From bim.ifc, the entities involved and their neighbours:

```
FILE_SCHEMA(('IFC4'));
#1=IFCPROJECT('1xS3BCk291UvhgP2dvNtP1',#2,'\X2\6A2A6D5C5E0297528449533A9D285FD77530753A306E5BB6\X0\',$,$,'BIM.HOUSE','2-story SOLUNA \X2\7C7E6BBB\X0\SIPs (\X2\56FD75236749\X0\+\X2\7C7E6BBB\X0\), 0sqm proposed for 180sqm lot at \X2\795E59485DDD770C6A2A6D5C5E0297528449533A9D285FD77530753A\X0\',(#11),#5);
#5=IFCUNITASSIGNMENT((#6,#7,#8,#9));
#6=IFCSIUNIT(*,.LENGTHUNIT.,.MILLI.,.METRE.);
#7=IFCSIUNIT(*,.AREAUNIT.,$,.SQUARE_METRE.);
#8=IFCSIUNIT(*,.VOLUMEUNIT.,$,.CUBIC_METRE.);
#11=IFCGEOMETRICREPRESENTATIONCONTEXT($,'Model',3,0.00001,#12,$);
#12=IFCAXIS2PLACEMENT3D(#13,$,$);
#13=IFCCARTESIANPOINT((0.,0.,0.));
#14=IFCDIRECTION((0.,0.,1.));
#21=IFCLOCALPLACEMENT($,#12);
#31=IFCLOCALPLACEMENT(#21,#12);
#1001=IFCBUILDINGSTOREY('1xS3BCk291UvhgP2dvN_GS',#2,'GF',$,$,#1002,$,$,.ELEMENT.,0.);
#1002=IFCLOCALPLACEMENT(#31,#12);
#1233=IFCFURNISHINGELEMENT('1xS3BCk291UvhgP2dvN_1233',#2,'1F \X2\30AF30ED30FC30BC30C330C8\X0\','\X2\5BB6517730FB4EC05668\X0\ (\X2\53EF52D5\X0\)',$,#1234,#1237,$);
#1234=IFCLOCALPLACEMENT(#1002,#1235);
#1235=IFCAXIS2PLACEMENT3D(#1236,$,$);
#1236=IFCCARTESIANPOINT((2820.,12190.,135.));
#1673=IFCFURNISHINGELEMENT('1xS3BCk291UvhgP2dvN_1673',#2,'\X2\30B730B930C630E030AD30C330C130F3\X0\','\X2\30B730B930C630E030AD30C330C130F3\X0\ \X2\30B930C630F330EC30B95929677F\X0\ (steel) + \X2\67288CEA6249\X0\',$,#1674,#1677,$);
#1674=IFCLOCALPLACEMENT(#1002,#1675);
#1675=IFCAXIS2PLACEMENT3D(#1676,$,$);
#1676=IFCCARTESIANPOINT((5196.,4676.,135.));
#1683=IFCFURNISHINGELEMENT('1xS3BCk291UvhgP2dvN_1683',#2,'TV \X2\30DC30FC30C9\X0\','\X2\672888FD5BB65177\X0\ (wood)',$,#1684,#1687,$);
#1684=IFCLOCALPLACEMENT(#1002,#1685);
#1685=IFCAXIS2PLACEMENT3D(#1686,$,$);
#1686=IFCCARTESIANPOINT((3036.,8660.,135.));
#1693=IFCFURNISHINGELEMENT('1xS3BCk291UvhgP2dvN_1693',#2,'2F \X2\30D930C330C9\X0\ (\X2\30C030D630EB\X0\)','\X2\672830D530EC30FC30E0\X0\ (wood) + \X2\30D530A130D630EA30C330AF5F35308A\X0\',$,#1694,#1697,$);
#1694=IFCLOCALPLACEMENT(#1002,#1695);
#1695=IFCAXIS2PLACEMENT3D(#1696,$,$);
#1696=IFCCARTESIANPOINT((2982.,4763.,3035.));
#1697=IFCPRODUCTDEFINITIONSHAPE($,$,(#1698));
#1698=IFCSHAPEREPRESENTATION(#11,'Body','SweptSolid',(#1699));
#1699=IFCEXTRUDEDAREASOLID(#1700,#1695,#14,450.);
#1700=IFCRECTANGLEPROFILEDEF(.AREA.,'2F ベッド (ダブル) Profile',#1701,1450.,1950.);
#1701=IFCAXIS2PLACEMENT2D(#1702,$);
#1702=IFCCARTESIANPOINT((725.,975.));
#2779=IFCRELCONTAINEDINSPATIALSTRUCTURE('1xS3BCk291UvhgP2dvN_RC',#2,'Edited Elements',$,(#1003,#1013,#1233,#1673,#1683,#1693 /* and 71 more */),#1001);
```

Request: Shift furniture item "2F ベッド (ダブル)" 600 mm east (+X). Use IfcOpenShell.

```python
import ifcopenshell
import ifcopenshell.api.geometry
import ifcopenshell.util.placement

model = ifcopenshell.open("bim.ifc")

item = model.by_id(1693)
matrix = ifcopenshell.util.placement.get_local_placement(item.ObjectPlacement)
matrix[0, 3] += 600.0
ifcopenshell.api.geometry.edit_object_placement(model, product=item, matrix=matrix, is_si=False)

print(ifcopenshell.util.placement.get_local_placement(item.ObjectPlacement).round(3) + 0.0)

model.write("bim_v2.ifc")
```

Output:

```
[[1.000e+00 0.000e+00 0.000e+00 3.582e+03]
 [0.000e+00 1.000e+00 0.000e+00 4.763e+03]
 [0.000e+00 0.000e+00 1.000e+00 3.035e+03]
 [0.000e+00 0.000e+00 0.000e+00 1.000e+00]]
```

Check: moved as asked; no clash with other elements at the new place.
